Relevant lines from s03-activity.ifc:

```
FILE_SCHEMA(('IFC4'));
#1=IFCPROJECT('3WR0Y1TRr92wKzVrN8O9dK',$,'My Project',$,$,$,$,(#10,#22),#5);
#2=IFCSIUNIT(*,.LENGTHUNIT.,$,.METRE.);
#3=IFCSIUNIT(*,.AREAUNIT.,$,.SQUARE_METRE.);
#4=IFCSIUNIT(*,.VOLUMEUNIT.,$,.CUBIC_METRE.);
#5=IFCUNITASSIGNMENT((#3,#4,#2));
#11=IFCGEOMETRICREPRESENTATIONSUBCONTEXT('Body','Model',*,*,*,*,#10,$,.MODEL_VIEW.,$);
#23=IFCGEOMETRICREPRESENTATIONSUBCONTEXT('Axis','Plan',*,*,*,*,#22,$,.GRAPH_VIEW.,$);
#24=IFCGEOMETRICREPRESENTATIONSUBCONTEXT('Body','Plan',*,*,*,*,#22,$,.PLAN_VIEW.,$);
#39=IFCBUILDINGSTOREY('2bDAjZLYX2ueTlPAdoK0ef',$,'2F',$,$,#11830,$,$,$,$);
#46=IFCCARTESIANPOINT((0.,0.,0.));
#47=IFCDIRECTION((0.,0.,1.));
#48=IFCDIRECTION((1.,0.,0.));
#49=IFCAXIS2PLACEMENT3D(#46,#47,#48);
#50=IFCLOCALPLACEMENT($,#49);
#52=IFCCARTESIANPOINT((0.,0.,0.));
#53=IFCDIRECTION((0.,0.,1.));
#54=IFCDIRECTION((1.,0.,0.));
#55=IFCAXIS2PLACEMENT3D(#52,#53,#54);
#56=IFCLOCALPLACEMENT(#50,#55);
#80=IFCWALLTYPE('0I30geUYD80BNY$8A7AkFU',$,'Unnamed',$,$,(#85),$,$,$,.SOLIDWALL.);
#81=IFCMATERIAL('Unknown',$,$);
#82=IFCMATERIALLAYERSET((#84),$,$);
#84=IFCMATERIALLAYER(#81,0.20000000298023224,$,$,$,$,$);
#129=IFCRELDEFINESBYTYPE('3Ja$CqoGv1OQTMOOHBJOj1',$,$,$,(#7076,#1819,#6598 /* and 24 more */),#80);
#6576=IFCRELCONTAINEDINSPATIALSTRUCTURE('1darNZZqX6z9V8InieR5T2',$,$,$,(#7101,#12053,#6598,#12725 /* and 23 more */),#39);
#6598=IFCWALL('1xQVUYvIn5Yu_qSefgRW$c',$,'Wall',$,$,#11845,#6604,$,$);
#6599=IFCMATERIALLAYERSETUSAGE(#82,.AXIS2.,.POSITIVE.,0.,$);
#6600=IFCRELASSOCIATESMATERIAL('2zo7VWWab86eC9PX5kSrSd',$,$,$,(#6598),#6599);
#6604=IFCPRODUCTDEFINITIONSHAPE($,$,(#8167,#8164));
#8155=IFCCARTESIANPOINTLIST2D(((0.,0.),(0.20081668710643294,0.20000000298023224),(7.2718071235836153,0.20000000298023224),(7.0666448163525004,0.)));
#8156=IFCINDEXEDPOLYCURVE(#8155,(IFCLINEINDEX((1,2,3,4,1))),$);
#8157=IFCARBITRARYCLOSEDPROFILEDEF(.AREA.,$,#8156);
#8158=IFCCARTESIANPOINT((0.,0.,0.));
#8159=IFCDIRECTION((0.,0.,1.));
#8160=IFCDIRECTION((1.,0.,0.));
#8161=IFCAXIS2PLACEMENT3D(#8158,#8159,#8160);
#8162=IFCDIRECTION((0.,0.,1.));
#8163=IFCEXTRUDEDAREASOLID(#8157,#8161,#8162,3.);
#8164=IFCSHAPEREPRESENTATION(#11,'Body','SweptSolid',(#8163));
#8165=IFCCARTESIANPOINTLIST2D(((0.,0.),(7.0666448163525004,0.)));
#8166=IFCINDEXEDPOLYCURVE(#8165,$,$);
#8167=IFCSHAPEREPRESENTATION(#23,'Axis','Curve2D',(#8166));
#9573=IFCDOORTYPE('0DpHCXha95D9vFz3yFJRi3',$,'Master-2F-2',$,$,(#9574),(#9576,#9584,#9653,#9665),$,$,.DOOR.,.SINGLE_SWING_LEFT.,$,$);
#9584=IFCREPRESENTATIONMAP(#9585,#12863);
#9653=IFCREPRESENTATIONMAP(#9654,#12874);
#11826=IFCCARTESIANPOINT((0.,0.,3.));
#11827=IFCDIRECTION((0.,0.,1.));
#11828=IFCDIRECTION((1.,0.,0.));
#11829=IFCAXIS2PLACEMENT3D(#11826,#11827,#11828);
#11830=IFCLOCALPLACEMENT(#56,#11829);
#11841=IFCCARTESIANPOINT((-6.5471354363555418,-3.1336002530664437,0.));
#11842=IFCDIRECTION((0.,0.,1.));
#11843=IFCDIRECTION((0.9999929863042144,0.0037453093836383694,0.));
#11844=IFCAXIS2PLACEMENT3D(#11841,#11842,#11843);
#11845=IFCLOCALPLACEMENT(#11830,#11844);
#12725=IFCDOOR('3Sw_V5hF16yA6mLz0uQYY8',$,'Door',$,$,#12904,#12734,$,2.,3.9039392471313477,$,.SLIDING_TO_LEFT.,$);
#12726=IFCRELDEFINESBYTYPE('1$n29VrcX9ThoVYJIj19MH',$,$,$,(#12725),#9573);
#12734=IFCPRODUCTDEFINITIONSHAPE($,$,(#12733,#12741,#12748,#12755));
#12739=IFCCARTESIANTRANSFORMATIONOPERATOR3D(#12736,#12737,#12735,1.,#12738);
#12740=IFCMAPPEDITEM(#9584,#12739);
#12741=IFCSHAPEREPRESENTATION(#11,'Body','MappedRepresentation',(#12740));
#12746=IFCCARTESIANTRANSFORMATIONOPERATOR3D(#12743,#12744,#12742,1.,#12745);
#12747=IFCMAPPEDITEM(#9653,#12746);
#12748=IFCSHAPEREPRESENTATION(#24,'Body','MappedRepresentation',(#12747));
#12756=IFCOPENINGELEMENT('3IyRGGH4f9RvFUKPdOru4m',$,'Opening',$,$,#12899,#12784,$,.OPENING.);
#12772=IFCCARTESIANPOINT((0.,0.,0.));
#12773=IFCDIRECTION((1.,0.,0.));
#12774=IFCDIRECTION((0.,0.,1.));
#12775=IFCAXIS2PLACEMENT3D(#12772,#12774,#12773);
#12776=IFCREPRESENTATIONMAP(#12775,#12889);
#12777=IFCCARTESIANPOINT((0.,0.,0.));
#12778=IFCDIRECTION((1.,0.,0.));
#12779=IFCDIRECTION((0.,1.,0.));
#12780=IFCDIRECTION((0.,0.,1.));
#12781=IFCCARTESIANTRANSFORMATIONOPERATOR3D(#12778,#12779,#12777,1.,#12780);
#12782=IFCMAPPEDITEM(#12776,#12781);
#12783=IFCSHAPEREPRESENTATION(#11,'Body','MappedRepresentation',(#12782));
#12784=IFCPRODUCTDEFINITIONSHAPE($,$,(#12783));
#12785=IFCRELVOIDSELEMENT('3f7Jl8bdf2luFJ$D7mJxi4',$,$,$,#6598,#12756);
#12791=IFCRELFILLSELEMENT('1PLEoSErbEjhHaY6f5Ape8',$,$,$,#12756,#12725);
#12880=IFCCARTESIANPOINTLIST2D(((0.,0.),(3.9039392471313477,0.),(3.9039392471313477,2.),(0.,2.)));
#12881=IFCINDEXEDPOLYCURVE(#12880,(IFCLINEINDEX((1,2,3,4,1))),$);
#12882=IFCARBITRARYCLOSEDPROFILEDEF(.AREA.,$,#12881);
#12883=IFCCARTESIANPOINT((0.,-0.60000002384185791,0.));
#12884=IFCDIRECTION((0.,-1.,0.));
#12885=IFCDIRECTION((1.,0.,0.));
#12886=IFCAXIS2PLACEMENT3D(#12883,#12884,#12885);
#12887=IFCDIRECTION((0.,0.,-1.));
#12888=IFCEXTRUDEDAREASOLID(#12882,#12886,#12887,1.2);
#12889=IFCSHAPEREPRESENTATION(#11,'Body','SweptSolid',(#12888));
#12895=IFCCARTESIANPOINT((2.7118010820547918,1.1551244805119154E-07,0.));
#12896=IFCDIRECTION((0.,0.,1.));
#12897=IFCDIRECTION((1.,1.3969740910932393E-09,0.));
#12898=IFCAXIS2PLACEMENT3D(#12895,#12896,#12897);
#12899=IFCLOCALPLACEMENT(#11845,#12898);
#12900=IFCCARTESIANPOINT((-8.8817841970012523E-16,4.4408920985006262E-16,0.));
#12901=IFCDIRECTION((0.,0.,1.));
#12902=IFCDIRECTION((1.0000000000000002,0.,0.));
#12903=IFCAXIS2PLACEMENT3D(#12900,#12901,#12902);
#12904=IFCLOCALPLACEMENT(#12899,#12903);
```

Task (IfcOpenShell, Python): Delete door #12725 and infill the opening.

```python
import ifcopenshell
import ifcopenshell.api.feature
import ifcopenshell.api.root
import ifcopenshell.geom
import ifcopenshell.util.shape

model = ifcopenshell.open("s03-activity.ifc")
settings = ifcopenshell.geom.settings()


def volume(element):
    """Net volume in cubic metres, openings subtracted."""
    shape = ifcopenshell.geom.create_shape(settings, element)
    return ifcopenshell.util.shape.get_volume(shape.geometry)


door = model.by_id(12725)
opening = door.FillsVoids[0].RelatingOpeningElement
wall = opening.VoidsElements[0].RelatingBuildingElement
before = volume(wall)

ifcopenshell.api.root.remove_product(model, product=door)
ifcopenshell.api.feature.remove_feature(model, feature=opening)

after = volume(wall)

print(f"wall volume {before:.3f} -> {after:.3f} m3")

model.write("s03-activity_v2.ifc")
```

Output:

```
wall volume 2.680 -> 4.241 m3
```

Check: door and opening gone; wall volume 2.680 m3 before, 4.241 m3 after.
